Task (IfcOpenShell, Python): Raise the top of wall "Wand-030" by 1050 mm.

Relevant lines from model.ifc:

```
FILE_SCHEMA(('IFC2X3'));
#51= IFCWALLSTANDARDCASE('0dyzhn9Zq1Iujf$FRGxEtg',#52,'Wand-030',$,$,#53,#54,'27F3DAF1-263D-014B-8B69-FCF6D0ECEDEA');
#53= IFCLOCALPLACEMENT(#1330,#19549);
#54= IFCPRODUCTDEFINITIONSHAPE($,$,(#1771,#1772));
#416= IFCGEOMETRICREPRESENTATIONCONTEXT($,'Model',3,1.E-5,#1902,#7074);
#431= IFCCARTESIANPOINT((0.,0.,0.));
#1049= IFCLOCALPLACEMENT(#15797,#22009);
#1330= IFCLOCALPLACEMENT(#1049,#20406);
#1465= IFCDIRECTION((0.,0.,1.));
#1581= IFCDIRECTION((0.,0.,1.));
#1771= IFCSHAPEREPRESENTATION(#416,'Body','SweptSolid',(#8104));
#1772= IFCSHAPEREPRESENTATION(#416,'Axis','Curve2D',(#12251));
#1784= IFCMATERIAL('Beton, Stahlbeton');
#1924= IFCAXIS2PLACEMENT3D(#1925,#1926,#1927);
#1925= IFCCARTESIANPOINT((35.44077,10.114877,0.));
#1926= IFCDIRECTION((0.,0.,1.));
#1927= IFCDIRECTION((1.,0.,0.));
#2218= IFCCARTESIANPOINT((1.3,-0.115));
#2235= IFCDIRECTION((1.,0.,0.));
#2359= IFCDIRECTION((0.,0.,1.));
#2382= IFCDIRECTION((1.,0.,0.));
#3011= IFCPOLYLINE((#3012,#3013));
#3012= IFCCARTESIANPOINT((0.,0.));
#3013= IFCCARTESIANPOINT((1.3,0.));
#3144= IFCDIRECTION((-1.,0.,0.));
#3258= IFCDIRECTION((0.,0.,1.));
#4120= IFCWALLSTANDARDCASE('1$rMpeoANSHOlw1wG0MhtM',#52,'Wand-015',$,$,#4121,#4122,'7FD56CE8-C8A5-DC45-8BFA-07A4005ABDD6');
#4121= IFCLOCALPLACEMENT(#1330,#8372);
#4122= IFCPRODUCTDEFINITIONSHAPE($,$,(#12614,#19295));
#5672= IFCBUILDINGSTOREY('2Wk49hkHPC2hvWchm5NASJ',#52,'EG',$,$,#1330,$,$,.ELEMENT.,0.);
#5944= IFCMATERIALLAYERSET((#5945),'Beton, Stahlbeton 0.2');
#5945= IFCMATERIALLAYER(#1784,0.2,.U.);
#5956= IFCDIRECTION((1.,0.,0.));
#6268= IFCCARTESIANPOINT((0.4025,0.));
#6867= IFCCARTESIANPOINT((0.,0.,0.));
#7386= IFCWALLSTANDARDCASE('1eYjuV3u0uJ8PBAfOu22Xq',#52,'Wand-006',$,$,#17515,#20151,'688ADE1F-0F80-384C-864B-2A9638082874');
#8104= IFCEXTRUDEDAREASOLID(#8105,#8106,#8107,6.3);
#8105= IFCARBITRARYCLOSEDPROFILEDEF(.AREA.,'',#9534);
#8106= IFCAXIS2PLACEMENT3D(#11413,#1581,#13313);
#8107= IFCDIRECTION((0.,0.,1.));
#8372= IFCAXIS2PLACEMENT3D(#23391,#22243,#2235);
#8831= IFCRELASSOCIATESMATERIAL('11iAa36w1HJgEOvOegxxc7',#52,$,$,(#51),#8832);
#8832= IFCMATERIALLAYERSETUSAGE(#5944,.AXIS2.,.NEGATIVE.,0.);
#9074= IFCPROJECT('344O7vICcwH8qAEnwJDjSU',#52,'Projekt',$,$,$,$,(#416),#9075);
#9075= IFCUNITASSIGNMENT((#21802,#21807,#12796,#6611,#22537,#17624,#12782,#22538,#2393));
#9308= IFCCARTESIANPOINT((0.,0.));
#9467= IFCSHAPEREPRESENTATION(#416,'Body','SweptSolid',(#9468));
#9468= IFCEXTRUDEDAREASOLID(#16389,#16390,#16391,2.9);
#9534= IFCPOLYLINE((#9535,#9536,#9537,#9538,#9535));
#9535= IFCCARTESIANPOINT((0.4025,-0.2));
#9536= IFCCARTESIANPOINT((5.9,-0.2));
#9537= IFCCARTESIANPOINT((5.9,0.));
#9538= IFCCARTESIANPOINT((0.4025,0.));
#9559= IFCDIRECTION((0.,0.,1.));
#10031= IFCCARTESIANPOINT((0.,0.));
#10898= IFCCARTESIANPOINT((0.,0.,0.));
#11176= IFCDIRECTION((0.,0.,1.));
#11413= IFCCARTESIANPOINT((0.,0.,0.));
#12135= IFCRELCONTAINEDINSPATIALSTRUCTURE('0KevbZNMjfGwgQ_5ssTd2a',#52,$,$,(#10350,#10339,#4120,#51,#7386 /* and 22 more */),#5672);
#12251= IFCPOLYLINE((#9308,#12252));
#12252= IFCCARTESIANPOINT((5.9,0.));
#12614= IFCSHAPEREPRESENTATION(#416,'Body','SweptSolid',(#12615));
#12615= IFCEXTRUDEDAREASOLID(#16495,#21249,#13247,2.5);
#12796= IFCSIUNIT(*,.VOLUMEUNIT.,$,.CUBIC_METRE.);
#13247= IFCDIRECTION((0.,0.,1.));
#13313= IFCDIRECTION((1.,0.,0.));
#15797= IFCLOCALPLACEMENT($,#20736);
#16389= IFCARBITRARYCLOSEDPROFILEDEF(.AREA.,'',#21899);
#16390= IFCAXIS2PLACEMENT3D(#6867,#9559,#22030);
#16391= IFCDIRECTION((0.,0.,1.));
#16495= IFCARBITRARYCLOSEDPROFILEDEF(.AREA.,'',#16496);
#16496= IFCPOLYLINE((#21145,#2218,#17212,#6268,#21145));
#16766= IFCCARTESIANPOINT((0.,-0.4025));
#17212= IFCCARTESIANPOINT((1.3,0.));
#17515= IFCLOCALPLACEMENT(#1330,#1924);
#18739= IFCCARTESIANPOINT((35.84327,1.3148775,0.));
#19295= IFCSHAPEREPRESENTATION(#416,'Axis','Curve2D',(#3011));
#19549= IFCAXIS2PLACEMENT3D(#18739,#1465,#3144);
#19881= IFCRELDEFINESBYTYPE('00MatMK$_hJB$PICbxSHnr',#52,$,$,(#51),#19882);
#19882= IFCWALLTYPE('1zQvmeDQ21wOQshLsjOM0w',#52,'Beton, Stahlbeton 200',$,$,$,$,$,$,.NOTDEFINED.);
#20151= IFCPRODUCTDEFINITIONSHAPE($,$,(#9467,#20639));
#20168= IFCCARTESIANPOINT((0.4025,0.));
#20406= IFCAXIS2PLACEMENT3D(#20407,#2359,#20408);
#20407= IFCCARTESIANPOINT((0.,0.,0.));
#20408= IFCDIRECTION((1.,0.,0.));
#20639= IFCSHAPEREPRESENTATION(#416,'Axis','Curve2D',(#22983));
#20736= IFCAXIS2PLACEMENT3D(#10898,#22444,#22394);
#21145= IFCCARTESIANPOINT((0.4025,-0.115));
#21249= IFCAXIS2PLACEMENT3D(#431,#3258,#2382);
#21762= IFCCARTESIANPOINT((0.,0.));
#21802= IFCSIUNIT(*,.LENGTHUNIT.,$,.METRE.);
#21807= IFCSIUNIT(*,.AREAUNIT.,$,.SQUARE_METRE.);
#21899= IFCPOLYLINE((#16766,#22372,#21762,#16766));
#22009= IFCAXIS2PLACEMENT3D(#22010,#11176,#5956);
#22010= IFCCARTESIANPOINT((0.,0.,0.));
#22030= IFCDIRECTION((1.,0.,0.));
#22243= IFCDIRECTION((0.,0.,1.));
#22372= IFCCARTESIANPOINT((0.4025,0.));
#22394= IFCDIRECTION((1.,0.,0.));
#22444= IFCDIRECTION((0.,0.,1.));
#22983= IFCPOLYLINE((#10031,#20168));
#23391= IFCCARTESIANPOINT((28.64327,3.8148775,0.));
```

```python
import ifcopenshell
import ifcopenshell.geom
import ifcopenshell.util.shape

model = ifcopenshell.open("model.ifc")
settings = ifcopenshell.geom.settings()


def volume(element):
    """Net volume in cubic metres, openings subtracted."""
    shape = ifcopenshell.geom.create_shape(settings, element)
    return ifcopenshell.util.shape.get_volume(shape.geometry)


wall = model.by_guid("0dyzhn9Zq1Iujf$FRGxEtg")
before = volume(wall)

body = next(r for r in wall.Representation.Representations if r.RepresentationIdentifier == "Body")
solid = body.Items[0]
old_height = solid.Depth
solid.Depth += 1.05
after = volume(wall)

print(f"height {old_height:g} -> {solid.Depth:g}, volume {before:.3f} -> {after:.3f} m3")

model.write("model-out.ifc")
```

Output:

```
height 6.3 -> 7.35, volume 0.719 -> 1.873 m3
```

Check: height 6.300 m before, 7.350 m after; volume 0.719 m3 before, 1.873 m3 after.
